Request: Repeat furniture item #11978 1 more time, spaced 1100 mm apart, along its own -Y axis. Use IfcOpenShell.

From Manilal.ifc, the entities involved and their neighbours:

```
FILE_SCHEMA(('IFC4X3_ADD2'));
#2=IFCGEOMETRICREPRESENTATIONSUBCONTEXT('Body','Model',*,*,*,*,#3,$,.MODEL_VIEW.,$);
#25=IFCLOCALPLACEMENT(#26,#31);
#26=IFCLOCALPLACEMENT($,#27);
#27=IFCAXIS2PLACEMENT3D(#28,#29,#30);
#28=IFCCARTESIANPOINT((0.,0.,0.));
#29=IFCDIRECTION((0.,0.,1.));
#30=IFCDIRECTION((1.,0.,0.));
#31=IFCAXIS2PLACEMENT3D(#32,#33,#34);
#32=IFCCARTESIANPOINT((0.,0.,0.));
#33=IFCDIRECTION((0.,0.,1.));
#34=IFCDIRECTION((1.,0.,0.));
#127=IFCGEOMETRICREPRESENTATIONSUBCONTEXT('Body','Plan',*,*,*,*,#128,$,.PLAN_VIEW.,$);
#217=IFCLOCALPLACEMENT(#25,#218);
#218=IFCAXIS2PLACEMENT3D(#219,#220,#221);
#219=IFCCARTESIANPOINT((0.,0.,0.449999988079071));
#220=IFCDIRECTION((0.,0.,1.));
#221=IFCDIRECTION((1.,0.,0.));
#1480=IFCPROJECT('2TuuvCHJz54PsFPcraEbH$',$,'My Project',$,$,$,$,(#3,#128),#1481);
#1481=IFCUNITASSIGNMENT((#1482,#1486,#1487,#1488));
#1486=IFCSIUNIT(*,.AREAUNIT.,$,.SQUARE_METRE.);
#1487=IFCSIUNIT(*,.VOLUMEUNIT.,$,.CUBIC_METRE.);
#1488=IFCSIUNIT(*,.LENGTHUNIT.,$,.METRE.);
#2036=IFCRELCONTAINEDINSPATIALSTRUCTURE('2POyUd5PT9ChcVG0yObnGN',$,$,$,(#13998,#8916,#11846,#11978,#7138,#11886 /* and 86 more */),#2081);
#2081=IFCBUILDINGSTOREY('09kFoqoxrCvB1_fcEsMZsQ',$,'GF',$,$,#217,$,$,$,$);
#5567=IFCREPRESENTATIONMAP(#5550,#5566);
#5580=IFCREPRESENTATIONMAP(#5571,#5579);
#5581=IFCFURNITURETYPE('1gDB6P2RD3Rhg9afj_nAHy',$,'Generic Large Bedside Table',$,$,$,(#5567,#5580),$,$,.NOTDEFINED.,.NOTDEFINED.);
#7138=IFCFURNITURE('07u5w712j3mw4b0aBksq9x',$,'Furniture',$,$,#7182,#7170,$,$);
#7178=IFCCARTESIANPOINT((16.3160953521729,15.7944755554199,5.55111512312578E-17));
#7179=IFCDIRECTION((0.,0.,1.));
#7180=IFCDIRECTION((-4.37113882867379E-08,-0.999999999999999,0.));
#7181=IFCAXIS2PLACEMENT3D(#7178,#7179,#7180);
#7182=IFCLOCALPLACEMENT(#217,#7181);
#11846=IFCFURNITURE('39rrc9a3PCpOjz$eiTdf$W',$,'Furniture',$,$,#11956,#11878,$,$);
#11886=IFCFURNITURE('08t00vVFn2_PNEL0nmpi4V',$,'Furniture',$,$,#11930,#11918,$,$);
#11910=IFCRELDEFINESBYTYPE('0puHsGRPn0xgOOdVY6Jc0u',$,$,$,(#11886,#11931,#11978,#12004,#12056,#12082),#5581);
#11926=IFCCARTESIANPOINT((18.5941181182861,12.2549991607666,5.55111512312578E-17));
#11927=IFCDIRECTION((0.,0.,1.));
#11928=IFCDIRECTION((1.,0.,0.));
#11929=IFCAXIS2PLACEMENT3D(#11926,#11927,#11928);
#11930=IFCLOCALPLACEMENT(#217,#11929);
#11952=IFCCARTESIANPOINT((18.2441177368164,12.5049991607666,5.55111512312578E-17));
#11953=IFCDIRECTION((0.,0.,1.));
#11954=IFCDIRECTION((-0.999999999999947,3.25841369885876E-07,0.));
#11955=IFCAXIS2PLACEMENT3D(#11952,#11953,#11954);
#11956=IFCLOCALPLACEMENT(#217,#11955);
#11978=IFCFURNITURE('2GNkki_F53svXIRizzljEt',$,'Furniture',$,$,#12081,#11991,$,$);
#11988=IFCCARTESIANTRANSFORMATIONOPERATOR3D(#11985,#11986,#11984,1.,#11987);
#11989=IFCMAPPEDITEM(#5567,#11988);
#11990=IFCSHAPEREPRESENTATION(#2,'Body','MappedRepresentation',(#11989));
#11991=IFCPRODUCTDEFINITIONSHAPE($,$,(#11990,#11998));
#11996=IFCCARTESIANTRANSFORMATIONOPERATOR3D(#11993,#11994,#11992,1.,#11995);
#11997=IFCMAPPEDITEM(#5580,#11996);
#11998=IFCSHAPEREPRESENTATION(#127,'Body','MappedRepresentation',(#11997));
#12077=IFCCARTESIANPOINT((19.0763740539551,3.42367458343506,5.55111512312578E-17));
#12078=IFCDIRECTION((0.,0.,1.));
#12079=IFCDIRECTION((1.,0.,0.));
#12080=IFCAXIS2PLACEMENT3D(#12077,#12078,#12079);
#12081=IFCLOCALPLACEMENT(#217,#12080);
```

```python
import ifcopenshell
import ifcopenshell.api.geometry
import ifcopenshell.api.root
import ifcopenshell.util.element
import ifcopenshell.util.placement

model = ifcopenshell.open("Manilal.ifc")

source = model.by_guid("2GNkki_F53svXIRizzljEt")
base = ifcopenshell.util.placement.get_local_placement(source.ObjectPlacement)
step = -base[:3, 1] * 1.1

for i in range(1, 2):
    copy = ifcopenshell.api.root.copy_class(model, product=source)
    copy.Representation = ifcopenshell.util.element.copy_deep(
        model, source.Representation, exclude=["IfcGeometricRepresentationContext", "IfcRepresentationMap"]
    )
    matrix = base.copy()
    matrix[:3, 3] += i * step
    print("added at", matrix[:3, 3].round(3) + 0.0)
    ifcopenshell.api.geometry.edit_object_placement(model, product=copy, matrix=matrix, is_si=False)

model.write("Manilal_rev.ifc")
```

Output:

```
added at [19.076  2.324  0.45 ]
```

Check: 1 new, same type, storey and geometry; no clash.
